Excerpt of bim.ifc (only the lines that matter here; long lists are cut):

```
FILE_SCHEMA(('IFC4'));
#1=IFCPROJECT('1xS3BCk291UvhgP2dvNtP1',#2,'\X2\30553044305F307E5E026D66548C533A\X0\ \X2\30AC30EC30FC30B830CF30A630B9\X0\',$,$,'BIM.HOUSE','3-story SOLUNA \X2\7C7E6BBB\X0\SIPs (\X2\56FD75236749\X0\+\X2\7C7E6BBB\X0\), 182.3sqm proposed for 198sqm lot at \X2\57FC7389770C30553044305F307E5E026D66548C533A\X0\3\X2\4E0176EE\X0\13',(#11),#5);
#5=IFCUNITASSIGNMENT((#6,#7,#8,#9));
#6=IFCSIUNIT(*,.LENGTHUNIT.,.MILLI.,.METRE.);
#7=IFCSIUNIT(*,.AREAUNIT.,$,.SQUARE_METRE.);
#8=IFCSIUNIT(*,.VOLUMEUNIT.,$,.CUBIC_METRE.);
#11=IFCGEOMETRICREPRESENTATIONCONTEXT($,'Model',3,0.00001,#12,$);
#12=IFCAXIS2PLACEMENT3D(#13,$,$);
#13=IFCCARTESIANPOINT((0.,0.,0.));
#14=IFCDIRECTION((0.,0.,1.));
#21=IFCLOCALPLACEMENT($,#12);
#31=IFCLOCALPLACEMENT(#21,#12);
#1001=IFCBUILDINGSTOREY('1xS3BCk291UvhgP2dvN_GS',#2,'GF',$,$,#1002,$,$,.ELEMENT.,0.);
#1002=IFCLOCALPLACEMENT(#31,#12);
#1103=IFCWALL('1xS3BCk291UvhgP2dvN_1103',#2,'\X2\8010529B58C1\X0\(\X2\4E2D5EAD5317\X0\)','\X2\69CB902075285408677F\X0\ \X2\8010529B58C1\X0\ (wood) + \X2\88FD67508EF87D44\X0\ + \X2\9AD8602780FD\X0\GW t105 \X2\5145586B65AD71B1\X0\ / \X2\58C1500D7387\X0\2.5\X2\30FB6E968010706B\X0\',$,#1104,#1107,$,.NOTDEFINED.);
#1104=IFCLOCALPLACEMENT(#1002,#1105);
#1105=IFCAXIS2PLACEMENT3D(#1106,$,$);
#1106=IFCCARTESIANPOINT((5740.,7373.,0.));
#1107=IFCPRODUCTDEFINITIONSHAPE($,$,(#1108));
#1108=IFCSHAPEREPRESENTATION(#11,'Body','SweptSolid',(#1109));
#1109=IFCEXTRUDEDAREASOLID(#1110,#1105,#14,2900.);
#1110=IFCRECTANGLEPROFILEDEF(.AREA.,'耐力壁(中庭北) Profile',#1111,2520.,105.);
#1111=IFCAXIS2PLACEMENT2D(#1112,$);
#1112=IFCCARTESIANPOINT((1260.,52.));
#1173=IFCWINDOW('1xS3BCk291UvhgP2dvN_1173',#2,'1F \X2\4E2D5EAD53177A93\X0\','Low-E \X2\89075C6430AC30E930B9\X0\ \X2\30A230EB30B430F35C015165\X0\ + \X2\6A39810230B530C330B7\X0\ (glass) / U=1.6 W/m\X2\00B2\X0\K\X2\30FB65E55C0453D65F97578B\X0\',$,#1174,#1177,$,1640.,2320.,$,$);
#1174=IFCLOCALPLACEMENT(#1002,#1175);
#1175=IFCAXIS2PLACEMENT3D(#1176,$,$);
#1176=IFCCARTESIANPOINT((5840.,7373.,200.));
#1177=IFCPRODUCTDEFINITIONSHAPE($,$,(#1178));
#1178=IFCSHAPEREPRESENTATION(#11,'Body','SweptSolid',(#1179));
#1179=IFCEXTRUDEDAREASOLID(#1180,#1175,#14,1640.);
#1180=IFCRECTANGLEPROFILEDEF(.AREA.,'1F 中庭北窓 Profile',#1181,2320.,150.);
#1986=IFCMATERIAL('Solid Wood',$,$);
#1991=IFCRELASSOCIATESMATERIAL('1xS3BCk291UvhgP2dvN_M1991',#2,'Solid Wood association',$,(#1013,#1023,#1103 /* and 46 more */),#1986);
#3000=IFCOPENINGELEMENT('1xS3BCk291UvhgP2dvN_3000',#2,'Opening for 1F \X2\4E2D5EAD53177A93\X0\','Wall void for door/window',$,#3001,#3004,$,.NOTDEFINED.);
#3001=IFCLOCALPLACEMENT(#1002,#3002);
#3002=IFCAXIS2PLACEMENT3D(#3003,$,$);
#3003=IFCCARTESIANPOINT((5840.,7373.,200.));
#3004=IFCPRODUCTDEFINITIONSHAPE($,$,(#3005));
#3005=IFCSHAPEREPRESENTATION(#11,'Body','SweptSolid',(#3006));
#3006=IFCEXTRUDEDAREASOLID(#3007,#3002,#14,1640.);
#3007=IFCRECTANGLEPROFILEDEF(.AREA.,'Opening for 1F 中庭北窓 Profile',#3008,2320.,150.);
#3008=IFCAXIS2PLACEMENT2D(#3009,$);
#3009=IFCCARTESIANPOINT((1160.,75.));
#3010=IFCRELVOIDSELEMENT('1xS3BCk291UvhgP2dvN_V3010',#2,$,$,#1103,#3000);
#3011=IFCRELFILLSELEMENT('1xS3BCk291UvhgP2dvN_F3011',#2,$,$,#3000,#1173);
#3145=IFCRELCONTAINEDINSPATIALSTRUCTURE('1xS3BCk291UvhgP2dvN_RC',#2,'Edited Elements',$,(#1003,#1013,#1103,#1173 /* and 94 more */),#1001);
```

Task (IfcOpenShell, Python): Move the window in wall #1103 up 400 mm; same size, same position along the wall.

```python
import numpy as np
import ifcopenshell
import ifcopenshell.api.geometry
import ifcopenshell.util.placement
import ifcopenshell.util.unit

model = ifcopenshell.open("bim.ifc")
unit_scale = ifcopenshell.util.unit.calculate_unit_scale(model)

window = model.by_guid("1xS3BCk291UvhgP2dvN_1173")
opening = window.FillsVoids[0].RelatingOpeningElement
dz = 0.4 / unit_scale

shift = np.array([0.0, 0.0, dz])
# The window is not placed relative to its opening, so move both.
for product in (opening, window):
    matrix = ifcopenshell.util.placement.get_local_placement(product.ObjectPlacement)
    matrix[:3, 3] += shift
    ifcopenshell.api.geometry.edit_object_placement(model, product=product, matrix=matrix, is_si=False)

print(f"moved by {dz * unit_scale:+.3f} m")

model.write("bim_v2.ifc")
```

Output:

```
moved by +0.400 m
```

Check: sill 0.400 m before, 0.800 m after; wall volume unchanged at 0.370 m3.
